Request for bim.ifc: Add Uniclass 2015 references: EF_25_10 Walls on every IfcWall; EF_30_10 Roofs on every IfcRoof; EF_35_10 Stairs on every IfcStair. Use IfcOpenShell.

First a look at what the model holds.

```python
import ifcopenshell

model = ifcopenshell.open("bim.ifc")
print(model.schema)
print("classifications:", [c.Name for c in model.by_type("IfcClassification")])
for ifc_class in ("IfcDoor", "IfcRoof", "IfcStair", "IfcWall", "IfcWindow"):
    print(ifc_class, len(model.by_type(ifc_class)))
```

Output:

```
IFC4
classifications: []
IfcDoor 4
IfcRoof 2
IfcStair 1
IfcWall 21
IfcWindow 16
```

```python
import ifcopenshell
import ifcopenshell.api.classification

model = ifcopenshell.open("bim.ifc")

system = ifcopenshell.api.classification.add_classification(model, classification="Uniclass 2015")

codes = {
    "IfcWall": ("EF_25_10", "Walls"),
    "IfcRoof": ("EF_30_10", "Roofs"),
    "IfcStair": ("EF_35_10", "Stairs"),
}
for ifc_class, (code, name) in codes.items():
    products = model.by_type(ifc_class)
    ifcopenshell.api.classification.add_reference(
        model, products=products, classification=system, identification=code, name=name
    )
    print(code, len(products))

model.write("bim_updated.ifc")
```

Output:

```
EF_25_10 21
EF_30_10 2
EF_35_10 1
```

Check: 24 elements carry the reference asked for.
